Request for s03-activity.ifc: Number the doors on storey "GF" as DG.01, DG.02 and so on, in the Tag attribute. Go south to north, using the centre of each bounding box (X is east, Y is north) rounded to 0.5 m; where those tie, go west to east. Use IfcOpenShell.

First a look at what the model holds.

```python
import ifcopenshell
import ifcopenshell.util.element
import ifcopenshell.util.placement

model = ifcopenshell.open("s03-activity.ifc")
print(model.schema)
storey = next(s for s in model.by_type("IfcBuildingStorey") if s.Name == "GF")
doors = [e for e in ifcopenshell.util.element.get_decomposition(storey) if e.is_a("IfcDoor")]
for e in sorted(doors, key=lambda e: e.id()):
    origin = ifcopenshell.util.placement.get_local_placement(e.ObjectPlacement)[:3, 3]
    print(e.id(), e.Tag, e.Name, origin.round(2) + 0.0, sep=" | ")
```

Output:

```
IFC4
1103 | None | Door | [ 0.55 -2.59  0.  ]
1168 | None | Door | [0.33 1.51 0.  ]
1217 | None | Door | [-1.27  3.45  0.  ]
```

```python
import ifcopenshell
import ifcopenshell.geom
import ifcopenshell.util.element
import ifcopenshell.util.shape

model = ifcopenshell.open("s03-activity.ifc")
settings = ifcopenshell.geom.settings()
settings.set("use-world-coords", True)


def centre(element):
    shape = ifcopenshell.geom.create_shape(settings, element)
    return ifcopenshell.util.shape.get_bbox_centroid(shape.geometry)


storey = next(s for s in model.by_type("IfcBuildingStorey") if s.Name == "GF")
doors = [e for e in ifcopenshell.util.element.get_decomposition(storey) if e.is_a("IfcDoor")]

# Insertion points can sit at a corner or the storey origin, so sort by the geometry (in metres).
centres = {e: centre(e) for e in doors}
doors.sort(key=lambda e: (round(centres[e][1] / 0.5), centres[e][0]))

for i, e in enumerate(doors, start=1):
    number = f"DG.{i:02d}"
    e.Tag = number
    print(e.id(), number)

model.write("s03-activity_updated.ifc")
```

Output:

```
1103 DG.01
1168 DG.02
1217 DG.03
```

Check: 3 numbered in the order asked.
